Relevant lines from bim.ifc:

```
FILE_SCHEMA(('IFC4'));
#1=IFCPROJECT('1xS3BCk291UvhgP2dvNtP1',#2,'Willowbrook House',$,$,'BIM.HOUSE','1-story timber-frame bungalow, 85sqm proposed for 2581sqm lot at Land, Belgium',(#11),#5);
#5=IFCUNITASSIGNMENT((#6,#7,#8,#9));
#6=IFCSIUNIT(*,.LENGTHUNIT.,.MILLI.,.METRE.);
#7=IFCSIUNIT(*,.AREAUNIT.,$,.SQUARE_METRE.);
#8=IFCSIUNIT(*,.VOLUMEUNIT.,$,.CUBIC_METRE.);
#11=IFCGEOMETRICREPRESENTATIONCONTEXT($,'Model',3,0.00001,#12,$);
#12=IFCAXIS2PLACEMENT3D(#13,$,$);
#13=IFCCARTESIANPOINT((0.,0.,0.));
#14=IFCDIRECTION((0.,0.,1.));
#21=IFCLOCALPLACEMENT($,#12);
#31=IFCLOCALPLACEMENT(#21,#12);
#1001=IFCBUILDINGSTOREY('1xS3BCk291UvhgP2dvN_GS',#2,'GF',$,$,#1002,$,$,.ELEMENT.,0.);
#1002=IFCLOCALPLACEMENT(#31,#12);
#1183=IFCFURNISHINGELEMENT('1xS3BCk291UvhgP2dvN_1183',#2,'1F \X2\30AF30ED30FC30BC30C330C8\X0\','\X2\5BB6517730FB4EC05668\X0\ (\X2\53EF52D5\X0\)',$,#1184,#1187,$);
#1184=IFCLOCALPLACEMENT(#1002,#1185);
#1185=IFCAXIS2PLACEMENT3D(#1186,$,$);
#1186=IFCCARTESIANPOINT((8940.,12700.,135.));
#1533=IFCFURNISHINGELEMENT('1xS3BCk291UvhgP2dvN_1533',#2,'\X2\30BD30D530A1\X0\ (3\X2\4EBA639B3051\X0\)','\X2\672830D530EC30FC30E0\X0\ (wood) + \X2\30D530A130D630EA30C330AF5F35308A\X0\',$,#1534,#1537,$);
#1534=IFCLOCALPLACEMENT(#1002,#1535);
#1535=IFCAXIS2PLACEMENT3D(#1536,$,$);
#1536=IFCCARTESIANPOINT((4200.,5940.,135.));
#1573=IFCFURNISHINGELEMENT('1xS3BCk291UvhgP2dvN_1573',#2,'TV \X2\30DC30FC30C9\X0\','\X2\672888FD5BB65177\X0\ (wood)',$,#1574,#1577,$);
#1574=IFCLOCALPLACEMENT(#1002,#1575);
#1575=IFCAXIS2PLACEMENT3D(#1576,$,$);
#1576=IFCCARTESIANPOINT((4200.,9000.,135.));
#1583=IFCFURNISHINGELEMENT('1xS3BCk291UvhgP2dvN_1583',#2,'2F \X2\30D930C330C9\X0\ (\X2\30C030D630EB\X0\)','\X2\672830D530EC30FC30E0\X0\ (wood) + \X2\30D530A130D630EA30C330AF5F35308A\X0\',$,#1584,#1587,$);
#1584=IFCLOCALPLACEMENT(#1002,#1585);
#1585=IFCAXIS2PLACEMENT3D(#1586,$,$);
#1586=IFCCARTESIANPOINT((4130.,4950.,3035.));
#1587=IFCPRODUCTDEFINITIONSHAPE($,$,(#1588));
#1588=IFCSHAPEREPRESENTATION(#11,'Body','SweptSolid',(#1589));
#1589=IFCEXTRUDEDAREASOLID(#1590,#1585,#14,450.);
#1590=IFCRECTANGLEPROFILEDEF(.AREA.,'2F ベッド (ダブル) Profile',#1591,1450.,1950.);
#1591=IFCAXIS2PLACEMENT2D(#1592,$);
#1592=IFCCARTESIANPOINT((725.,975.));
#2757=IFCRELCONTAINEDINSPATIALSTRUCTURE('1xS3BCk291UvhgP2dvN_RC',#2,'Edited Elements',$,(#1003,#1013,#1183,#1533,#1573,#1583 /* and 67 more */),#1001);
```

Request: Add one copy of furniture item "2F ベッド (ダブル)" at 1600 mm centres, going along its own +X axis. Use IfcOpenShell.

```python
import ifcopenshell
import ifcopenshell.api.geometry
import ifcopenshell.api.root
import ifcopenshell.util.element
import ifcopenshell.util.placement
import ifcopenshell.util.unit

model = ifcopenshell.open("bim.ifc")
unit_scale = ifcopenshell.util.unit.calculate_unit_scale(model)


def reuse_history(source, copy):
    """copy_class also copies each property set's owner history, people and application; keep the originals."""
    for rel in copy.IsDefinedBy:
        if rel.is_a("IfcRelDefinesByProperties") and (history := rel.RelatingPropertyDefinition.OwnerHistory):
            rel.RelatingPropertyDefinition.OwnerHistory = source.OwnerHistory
            ifcopenshell.util.element.remove_deep2(model, history)


source = model.by_id(1583)
base = ifcopenshell.util.placement.get_local_placement(source.ObjectPlacement)
step = base[:3, 0] * 1.6 / unit_scale

for i in range(1, 2):
    copy = ifcopenshell.api.root.copy_class(model, product=source)
    copy.Representation = ifcopenshell.util.element.copy_deep(
        model, source.Representation, exclude=["IfcGeometricRepresentationContext", "IfcRepresentationMap"]
    )
    reuse_history(source, copy)
    matrix = base.copy()
    matrix[:3, 3] += i * step
    print("added at", matrix[:3, 3].round(3) + 0.0)
    ifcopenshell.api.geometry.edit_object_placement(model, product=copy, matrix=matrix, is_si=False)

model.write("bim-out.ifc")
```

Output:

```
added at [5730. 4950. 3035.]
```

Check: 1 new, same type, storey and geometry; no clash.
